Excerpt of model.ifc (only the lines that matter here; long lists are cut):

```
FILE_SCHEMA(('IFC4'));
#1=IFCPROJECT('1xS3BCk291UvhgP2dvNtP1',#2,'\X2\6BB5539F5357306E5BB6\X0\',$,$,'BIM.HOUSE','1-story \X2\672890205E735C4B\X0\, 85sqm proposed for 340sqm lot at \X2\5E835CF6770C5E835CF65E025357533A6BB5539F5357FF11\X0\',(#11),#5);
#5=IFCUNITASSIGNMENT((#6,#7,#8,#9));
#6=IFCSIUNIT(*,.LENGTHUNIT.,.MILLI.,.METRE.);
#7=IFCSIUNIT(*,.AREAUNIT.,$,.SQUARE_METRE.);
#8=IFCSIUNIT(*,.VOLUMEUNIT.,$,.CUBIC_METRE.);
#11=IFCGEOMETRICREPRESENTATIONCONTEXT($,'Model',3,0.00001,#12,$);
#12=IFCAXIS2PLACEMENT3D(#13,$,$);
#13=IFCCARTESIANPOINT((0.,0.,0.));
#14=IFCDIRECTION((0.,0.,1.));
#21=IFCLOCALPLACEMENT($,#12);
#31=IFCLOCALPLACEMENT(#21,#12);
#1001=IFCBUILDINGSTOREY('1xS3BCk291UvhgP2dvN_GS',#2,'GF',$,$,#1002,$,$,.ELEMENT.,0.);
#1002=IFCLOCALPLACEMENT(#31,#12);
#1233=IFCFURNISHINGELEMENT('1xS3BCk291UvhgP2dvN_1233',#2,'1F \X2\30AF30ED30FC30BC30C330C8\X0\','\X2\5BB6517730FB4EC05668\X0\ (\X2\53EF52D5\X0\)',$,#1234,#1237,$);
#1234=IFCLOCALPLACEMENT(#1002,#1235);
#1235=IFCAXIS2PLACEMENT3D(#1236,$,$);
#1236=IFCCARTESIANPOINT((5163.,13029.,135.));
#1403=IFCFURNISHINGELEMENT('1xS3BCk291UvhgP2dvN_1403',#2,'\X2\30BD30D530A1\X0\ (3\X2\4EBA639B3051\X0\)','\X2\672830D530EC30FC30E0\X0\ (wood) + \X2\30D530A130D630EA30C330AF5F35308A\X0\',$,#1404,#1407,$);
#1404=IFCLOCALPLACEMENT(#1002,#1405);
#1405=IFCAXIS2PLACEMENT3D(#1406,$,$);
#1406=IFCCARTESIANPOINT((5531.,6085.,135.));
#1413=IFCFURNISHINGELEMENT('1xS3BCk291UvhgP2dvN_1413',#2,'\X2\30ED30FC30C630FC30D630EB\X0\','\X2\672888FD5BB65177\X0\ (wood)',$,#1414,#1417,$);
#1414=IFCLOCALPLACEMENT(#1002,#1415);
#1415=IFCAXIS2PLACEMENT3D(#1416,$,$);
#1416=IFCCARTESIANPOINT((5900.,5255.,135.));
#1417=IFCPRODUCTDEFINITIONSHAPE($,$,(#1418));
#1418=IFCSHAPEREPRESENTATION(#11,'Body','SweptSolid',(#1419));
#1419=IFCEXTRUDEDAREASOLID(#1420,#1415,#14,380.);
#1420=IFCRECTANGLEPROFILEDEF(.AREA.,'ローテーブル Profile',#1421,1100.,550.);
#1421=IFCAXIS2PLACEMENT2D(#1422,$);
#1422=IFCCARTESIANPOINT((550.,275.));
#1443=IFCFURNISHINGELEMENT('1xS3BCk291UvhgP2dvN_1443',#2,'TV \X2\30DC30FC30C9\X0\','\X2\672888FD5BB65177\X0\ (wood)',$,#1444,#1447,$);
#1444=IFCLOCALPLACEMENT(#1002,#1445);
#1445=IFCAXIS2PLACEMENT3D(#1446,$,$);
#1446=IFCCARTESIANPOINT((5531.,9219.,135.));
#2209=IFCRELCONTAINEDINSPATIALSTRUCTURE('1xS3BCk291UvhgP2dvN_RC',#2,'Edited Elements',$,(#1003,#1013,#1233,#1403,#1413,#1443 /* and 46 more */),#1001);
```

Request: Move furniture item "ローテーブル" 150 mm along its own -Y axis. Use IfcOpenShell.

```python
import ifcopenshell
import ifcopenshell.api.geometry
import ifcopenshell.util.placement
import ifcopenshell.util.unit

model = ifcopenshell.open("model.ifc")
unit_scale = ifcopenshell.util.unit.calculate_unit_scale(model)

item = model.by_guid("1xS3BCk291UvhgP2dvN_1413")
matrix = ifcopenshell.util.placement.get_local_placement(item.ObjectPlacement)
matrix[:3, 3] -= matrix[:3, 1] * 0.15 / unit_scale
ifcopenshell.api.geometry.edit_object_placement(model, product=item, matrix=matrix, is_si=False)

print(ifcopenshell.util.placement.get_local_placement(item.ObjectPlacement).round(3) + 0.0)

model.write("model-out.ifc")
```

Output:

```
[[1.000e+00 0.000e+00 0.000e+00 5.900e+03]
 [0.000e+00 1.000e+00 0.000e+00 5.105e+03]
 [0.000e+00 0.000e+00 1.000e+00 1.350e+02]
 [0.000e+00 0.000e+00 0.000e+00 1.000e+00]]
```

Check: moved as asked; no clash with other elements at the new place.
